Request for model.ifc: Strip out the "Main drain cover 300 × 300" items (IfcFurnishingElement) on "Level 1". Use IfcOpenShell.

First a look at what the model holds.

```python
import ifcopenshell
import ifcopenshell.util.element

model = ifcopenshell.open("model.ifc")
print(model.schema)
storey = next(s for s in model.by_type("IfcBuildingStorey") if s.Name == "Level 1")
furniture = [e for e in ifcopenshell.util.element.get_decomposition(storey) if e.is_a("IfcFurnishingElement")]
seen = {}
for e in furniture:
    element_type = ifcopenshell.util.element.get_type(e)
    name = element_type.Name if element_type not in (None, e) else None
    seen[name] = seen.get(name, 0) + 1
for name, count in sorted(seen.items(), key=str):
    print(count, "x", name)
```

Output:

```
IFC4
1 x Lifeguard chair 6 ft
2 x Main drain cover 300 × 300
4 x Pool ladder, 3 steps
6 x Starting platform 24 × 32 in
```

```python
import ifcopenshell
import ifcopenshell.api.root
import ifcopenshell.util.element

model = ifcopenshell.open("model.ifc")

storey = next(s for s in model.by_type("IfcBuildingStorey") if s.Name == "Level 1")
furniture = [e for e in ifcopenshell.util.element.get_decomposition(storey) if e.is_a("IfcFurnishingElement")]
targets = [e for e in furniture if (t := ifcopenshell.util.element.get_type(e)) not in (None, e) and t.Name == "Main drain cover 300 × 300"]

for e in targets:
    ifcopenshell.api.root.remove_product(model, product=e)
print(len(targets), "removed")

model.write("model-out.ifc")
```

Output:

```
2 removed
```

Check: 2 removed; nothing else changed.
